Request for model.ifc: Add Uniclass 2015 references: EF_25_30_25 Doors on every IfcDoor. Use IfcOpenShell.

First a look at what the model holds.

```python
import ifcopenshell

model = ifcopenshell.open("model.ifc")
print(model.schema)
print("classifications:", [c.Name for c in model.by_type("IfcClassification")])
for ifc_class in ("IfcDoor", "IfcRoof", "IfcStair", "IfcWall", "IfcWindow"):
    print(ifc_class, len(model.by_type(ifc_class)))
```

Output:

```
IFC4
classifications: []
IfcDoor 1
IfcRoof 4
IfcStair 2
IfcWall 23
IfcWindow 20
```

```python
import ifcopenshell
import ifcopenshell.api.classification

model = ifcopenshell.open("model.ifc")

system = ifcopenshell.api.classification.add_classification(model, classification="Uniclass 2015")

codes = {
    "IfcDoor": ("EF_25_30_25", "Doors"),
}
for ifc_class, (code, name) in codes.items():
    products = model.by_type(ifc_class)
    ifcopenshell.api.classification.add_reference(
        model, products=products, classification=system, identification=code, name=name
    )
    print(code, len(products))

model.write("model_rev.ifc")
```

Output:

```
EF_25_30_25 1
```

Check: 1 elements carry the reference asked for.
